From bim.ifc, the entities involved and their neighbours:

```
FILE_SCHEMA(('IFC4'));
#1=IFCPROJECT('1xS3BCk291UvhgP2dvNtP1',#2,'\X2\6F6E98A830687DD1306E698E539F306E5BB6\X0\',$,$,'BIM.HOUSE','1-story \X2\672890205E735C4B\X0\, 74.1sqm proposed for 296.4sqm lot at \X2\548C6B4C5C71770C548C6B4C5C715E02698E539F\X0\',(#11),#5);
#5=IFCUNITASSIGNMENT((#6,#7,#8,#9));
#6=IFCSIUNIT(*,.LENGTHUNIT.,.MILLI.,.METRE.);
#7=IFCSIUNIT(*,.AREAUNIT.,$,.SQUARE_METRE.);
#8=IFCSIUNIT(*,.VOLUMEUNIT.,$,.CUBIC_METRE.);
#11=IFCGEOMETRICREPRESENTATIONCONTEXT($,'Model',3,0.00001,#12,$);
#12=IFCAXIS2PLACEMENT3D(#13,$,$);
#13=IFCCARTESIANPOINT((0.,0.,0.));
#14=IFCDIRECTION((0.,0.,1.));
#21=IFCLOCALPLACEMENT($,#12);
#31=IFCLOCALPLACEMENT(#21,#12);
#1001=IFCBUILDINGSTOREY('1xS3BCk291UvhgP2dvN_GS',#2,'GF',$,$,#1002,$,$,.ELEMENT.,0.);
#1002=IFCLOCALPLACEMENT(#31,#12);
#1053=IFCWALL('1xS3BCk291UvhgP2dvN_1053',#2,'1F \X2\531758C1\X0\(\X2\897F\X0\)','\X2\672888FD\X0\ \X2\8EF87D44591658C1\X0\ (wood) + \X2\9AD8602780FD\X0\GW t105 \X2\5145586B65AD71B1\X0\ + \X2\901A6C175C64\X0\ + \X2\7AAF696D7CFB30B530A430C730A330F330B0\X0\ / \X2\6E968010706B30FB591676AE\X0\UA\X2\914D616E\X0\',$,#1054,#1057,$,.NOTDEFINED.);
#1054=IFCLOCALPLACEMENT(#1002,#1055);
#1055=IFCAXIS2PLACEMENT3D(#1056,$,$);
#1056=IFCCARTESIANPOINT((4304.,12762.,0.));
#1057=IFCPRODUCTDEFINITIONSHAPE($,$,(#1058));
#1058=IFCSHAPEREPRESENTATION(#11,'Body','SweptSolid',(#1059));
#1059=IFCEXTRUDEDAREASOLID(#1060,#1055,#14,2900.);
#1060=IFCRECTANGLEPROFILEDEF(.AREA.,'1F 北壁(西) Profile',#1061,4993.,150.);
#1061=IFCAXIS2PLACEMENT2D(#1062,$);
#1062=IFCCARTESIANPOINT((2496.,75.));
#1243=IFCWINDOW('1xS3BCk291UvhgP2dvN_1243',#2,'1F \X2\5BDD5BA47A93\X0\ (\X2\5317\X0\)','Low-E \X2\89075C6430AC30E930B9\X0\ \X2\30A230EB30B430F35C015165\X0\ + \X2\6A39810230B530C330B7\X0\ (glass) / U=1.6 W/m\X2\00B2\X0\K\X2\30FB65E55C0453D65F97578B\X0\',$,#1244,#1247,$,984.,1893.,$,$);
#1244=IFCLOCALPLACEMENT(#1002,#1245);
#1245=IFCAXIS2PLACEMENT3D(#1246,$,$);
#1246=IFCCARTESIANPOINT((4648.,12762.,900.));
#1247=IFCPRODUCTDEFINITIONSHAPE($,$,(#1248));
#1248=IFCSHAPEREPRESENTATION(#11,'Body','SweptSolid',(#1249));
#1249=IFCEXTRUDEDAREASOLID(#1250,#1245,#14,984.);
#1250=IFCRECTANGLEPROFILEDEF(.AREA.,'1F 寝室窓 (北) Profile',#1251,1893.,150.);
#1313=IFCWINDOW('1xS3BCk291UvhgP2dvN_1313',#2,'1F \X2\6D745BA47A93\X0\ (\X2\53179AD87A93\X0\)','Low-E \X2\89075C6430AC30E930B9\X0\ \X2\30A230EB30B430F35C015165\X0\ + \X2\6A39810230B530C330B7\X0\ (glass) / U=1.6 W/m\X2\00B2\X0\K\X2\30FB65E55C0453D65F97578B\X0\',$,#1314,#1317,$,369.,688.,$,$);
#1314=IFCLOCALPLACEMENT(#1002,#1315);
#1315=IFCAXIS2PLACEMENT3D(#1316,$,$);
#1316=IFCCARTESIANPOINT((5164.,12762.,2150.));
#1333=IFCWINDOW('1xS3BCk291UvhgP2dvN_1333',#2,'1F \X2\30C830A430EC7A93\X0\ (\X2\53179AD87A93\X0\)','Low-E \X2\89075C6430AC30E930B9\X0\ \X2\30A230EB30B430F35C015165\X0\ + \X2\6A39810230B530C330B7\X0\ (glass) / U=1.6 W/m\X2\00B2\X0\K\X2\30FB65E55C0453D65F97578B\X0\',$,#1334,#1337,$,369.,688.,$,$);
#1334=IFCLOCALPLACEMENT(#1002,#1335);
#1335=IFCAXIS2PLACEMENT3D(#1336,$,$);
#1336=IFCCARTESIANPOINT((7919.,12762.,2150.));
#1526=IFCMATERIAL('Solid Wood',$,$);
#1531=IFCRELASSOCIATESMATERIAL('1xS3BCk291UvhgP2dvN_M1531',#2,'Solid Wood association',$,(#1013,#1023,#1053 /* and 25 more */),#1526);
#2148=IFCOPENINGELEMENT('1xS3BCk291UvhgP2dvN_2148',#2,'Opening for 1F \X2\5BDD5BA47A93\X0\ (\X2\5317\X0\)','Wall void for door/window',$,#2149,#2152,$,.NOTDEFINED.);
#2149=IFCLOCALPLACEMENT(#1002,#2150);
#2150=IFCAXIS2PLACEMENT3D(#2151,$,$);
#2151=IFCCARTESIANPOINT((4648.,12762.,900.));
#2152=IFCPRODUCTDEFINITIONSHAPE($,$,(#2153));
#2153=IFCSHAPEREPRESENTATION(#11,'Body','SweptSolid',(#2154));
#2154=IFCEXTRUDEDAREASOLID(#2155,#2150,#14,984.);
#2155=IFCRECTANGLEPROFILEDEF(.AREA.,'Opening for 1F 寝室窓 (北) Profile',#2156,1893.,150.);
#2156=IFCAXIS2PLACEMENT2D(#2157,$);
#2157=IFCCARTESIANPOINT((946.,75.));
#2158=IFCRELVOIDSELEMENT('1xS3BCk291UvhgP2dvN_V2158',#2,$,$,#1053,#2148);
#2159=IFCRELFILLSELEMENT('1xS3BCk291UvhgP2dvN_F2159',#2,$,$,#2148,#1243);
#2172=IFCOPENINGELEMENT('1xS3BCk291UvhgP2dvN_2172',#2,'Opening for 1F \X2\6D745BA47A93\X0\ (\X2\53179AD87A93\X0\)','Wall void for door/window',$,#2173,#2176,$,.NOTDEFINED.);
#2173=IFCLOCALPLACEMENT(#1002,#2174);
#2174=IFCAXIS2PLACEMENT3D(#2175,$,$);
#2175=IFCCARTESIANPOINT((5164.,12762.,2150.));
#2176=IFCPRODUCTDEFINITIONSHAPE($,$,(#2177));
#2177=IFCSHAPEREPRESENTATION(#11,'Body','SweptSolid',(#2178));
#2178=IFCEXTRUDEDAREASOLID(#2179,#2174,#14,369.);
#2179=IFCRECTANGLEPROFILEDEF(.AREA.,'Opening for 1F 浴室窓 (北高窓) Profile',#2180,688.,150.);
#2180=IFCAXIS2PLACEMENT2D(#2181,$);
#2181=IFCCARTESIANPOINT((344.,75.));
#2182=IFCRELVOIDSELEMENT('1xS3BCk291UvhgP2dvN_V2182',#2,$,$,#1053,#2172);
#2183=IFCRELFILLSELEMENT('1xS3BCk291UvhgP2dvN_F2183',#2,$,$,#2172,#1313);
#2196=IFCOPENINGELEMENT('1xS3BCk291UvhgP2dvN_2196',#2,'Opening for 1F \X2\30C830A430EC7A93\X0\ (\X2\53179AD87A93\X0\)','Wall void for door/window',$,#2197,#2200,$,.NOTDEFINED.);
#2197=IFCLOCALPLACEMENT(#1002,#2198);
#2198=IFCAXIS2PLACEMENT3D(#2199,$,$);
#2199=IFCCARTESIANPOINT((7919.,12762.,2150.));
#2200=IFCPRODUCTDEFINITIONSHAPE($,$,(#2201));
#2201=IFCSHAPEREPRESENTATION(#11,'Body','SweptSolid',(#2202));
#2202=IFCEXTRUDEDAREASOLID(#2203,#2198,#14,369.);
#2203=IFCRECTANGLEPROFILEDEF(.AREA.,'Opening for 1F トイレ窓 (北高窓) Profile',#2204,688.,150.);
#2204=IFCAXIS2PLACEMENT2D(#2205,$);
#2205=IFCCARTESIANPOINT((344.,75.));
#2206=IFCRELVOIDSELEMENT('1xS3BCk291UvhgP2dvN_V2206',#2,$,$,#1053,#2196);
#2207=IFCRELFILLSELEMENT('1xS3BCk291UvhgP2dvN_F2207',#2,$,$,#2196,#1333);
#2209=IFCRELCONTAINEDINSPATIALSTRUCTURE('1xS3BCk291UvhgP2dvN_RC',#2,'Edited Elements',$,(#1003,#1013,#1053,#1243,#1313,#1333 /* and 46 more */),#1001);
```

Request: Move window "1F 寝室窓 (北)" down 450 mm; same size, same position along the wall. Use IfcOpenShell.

```python
import numpy as np
import ifcopenshell
import ifcopenshell.api.geometry
import ifcopenshell.util.placement
import ifcopenshell.util.unit

model = ifcopenshell.open("bim.ifc")
unit_scale = ifcopenshell.util.unit.calculate_unit_scale(model)

window = model.by_guid("1xS3BCk291UvhgP2dvN_1243")
opening = window.FillsVoids[0].RelatingOpeningElement
dz = -0.45 / unit_scale

shift = np.array([0.0, 0.0, dz])
# The window is not placed relative to its opening, so move both.
for product in (opening, window):
    matrix = ifcopenshell.util.placement.get_local_placement(product.ObjectPlacement)
    matrix[:3, 3] += shift
    ifcopenshell.api.geometry.edit_object_placement(model, product=product, matrix=matrix, is_si=False)

print(f"moved by {dz * unit_scale:+.3f} m")

model.write("bim_updated.ifc")
```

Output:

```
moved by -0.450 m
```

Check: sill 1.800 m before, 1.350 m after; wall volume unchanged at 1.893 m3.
